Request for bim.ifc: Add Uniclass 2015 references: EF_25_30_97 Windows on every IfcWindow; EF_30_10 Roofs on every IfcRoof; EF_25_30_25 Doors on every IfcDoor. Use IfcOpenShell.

First a look at what the model holds.

```python
import ifcopenshell

model = ifcopenshell.open("bim.ifc")
print(model.schema)
print("classifications:", [c.Name for c in model.by_type("IfcClassification")])
for ifc_class in ("IfcDoor", "IfcRoof", "IfcStair", "IfcWall", "IfcWindow"):
    print(ifc_class, len(model.by_type(ifc_class)))
```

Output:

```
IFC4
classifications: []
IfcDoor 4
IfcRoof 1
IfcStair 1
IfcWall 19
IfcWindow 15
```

```python
import ifcopenshell
import ifcopenshell.api.classification

model = ifcopenshell.open("bim.ifc")

system = ifcopenshell.api.classification.add_classification(model, classification="Uniclass 2015")

codes = {
    "IfcWindow": ("EF_25_30_97", "Windows"),
    "IfcRoof": ("EF_30_10", "Roofs"),
    "IfcDoor": ("EF_25_30_25", "Doors"),
}
for ifc_class, (code, name) in codes.items():
    products = model.by_type(ifc_class)
    ifcopenshell.api.classification.add_reference(
        model, products=products, classification=system, identification=code, name=name
    )
    print(code, len(products))

model.write("bim_edited.ifc")
```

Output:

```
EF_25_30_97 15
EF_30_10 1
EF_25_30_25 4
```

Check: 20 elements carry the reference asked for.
